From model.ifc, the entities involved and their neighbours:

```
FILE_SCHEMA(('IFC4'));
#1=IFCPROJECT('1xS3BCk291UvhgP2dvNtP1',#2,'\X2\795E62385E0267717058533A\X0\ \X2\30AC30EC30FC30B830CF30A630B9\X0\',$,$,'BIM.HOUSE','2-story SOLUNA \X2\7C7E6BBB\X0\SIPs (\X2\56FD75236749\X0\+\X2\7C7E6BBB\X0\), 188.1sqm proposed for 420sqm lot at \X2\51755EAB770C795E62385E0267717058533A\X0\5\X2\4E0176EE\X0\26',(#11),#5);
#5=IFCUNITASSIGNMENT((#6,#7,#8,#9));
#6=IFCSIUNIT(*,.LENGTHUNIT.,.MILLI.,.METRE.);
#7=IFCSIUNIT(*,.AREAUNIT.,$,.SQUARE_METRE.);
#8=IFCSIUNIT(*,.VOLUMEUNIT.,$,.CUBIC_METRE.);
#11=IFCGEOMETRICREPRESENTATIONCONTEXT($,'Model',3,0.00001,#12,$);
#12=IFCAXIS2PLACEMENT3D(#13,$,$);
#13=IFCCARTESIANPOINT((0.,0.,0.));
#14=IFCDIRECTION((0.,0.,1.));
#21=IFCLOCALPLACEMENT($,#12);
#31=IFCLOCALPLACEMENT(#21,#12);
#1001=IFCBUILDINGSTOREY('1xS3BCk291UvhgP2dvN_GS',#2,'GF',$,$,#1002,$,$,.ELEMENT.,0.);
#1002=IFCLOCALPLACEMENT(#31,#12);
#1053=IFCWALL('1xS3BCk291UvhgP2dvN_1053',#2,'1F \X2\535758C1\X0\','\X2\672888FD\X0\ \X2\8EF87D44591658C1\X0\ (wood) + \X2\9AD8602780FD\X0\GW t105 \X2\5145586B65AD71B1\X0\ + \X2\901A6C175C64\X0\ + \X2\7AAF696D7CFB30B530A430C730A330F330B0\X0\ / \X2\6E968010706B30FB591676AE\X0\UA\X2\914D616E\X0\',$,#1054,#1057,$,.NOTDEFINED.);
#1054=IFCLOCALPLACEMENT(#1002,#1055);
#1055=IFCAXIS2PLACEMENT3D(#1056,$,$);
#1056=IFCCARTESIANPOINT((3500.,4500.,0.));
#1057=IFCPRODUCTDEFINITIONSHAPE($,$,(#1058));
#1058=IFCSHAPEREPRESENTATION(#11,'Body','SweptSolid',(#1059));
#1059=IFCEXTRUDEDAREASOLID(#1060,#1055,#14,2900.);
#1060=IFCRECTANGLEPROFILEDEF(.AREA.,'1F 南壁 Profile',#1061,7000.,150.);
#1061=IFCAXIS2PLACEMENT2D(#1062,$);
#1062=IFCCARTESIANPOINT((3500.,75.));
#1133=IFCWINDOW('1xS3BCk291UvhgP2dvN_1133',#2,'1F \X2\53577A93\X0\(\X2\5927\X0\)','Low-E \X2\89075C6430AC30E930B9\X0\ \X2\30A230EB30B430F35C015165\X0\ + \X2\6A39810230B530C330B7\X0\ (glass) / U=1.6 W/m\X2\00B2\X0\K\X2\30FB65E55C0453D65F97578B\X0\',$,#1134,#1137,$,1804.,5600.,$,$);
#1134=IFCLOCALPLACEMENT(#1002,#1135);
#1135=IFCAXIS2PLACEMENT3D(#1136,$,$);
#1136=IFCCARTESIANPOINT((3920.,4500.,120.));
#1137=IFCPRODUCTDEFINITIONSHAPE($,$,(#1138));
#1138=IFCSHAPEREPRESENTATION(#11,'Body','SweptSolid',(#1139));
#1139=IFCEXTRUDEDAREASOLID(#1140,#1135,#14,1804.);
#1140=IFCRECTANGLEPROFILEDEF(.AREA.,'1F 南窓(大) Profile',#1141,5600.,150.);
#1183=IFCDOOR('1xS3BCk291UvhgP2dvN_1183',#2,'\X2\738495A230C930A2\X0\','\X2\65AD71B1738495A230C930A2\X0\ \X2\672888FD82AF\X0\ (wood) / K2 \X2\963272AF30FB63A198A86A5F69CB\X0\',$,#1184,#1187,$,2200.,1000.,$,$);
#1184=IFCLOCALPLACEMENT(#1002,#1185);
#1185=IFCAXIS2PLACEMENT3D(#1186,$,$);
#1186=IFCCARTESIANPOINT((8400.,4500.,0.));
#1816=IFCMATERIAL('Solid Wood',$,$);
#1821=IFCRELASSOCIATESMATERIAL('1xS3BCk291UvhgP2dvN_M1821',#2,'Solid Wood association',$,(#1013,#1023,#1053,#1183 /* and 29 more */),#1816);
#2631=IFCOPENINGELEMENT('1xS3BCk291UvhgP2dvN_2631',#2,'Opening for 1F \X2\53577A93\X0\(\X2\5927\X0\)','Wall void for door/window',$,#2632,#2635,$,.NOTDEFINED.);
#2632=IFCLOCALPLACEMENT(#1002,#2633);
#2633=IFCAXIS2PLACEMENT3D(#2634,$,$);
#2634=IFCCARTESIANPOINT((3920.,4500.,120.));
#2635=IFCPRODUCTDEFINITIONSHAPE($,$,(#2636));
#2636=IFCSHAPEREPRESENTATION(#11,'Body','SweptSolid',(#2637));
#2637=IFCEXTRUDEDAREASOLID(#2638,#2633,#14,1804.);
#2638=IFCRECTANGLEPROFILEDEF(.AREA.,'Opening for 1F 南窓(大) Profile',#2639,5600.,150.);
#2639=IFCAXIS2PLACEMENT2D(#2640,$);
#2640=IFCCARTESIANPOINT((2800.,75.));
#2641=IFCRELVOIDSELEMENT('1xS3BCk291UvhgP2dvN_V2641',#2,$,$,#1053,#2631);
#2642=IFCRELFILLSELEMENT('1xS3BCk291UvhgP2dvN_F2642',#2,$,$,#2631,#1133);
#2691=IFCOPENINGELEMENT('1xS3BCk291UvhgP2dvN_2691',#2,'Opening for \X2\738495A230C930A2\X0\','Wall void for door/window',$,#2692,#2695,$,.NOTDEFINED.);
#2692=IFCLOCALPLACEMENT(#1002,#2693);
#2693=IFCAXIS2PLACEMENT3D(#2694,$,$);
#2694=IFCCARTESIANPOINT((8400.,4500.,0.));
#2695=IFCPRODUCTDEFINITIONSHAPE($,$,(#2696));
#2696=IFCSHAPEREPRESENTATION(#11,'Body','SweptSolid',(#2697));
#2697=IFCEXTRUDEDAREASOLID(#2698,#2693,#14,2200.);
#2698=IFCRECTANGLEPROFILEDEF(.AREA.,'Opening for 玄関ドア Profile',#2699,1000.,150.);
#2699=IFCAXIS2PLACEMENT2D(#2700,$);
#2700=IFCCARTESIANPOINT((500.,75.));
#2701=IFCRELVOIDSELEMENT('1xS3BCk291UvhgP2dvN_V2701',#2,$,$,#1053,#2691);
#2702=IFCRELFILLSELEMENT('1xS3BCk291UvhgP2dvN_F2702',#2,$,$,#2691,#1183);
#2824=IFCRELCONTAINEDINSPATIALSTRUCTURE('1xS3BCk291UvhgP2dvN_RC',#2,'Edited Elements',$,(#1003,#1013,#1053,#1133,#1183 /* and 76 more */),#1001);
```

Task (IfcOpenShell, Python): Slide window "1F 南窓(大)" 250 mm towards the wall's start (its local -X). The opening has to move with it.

```python
import ifcopenshell
import ifcopenshell.api.geometry
import ifcopenshell.util.placement
import ifcopenshell.util.unit

model = ifcopenshell.open("model.ifc")
unit_scale = ifcopenshell.util.unit.calculate_unit_scale(model)

window = model.by_guid("1xS3BCk291UvhgP2dvN_1133")
opening = window.FillsVoids[0].RelatingOpeningElement
wall = opening.VoidsElements[0].RelatingBuildingElement

wall_matrix = ifcopenshell.util.placement.get_local_placement(wall.ObjectPlacement)
shift = wall_matrix[:3, 0] * -0.25 / unit_scale
before = ifcopenshell.util.placement.get_local_placement(window.ObjectPlacement)[:3, 3].copy()

# The window is not placed relative to its opening, so move both.
for product in (opening, window):
    matrix = ifcopenshell.util.placement.get_local_placement(product.ObjectPlacement)
    matrix[:3, 3] += shift
    ifcopenshell.api.geometry.edit_object_placement(model, product=product, matrix=matrix, is_si=False)

after = ifcopenshell.util.placement.get_local_placement(window.ObjectPlacement)[:3, 3]
print("window moved by", (after - before).round(3) + 0.0)

model.write("model_v2.ifc")
```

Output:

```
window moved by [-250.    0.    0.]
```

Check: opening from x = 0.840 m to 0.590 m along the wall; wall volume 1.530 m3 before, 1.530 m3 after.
